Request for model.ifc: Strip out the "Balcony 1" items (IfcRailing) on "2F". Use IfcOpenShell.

First a look at what the model holds.

```python
import ifcopenshell
import ifcopenshell.util.element

model = ifcopenshell.open("model.ifc")
print(model.schema)
storey = next(s for s in model.by_type("IfcBuildingStorey") if s.Name == "2F")
railings = [e for e in ifcopenshell.util.element.get_decomposition(storey) if e.is_a("IfcRailing")]
seen = {}
for e in railings:
    element_type = ifcopenshell.util.element.get_type(e)
    name = element_type.Name if element_type not in (None, e) else None
    seen[name] = seen.get(name, 0) + 1
for name, count in sorted(seen.items(), key=str):
    print(count, "x", name)
```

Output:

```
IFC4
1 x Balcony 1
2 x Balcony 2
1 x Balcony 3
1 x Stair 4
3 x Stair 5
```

```python
import ifcopenshell
import ifcopenshell.api.root
import ifcopenshell.util.element

model = ifcopenshell.open("model.ifc")

storey = next(s for s in model.by_type("IfcBuildingStorey") if s.Name == "2F")
railings = [e for e in ifcopenshell.util.element.get_decomposition(storey) if e.is_a("IfcRailing")]
targets = [e for e in railings if (t := ifcopenshell.util.element.get_type(e)) not in (None, e) and t.Name == "Balcony 1"]

for e in targets:
    ifcopenshell.api.root.remove_product(model, product=e)
print(len(targets), "removed")

model.write("model_edited.ifc")
```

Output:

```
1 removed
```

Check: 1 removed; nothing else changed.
